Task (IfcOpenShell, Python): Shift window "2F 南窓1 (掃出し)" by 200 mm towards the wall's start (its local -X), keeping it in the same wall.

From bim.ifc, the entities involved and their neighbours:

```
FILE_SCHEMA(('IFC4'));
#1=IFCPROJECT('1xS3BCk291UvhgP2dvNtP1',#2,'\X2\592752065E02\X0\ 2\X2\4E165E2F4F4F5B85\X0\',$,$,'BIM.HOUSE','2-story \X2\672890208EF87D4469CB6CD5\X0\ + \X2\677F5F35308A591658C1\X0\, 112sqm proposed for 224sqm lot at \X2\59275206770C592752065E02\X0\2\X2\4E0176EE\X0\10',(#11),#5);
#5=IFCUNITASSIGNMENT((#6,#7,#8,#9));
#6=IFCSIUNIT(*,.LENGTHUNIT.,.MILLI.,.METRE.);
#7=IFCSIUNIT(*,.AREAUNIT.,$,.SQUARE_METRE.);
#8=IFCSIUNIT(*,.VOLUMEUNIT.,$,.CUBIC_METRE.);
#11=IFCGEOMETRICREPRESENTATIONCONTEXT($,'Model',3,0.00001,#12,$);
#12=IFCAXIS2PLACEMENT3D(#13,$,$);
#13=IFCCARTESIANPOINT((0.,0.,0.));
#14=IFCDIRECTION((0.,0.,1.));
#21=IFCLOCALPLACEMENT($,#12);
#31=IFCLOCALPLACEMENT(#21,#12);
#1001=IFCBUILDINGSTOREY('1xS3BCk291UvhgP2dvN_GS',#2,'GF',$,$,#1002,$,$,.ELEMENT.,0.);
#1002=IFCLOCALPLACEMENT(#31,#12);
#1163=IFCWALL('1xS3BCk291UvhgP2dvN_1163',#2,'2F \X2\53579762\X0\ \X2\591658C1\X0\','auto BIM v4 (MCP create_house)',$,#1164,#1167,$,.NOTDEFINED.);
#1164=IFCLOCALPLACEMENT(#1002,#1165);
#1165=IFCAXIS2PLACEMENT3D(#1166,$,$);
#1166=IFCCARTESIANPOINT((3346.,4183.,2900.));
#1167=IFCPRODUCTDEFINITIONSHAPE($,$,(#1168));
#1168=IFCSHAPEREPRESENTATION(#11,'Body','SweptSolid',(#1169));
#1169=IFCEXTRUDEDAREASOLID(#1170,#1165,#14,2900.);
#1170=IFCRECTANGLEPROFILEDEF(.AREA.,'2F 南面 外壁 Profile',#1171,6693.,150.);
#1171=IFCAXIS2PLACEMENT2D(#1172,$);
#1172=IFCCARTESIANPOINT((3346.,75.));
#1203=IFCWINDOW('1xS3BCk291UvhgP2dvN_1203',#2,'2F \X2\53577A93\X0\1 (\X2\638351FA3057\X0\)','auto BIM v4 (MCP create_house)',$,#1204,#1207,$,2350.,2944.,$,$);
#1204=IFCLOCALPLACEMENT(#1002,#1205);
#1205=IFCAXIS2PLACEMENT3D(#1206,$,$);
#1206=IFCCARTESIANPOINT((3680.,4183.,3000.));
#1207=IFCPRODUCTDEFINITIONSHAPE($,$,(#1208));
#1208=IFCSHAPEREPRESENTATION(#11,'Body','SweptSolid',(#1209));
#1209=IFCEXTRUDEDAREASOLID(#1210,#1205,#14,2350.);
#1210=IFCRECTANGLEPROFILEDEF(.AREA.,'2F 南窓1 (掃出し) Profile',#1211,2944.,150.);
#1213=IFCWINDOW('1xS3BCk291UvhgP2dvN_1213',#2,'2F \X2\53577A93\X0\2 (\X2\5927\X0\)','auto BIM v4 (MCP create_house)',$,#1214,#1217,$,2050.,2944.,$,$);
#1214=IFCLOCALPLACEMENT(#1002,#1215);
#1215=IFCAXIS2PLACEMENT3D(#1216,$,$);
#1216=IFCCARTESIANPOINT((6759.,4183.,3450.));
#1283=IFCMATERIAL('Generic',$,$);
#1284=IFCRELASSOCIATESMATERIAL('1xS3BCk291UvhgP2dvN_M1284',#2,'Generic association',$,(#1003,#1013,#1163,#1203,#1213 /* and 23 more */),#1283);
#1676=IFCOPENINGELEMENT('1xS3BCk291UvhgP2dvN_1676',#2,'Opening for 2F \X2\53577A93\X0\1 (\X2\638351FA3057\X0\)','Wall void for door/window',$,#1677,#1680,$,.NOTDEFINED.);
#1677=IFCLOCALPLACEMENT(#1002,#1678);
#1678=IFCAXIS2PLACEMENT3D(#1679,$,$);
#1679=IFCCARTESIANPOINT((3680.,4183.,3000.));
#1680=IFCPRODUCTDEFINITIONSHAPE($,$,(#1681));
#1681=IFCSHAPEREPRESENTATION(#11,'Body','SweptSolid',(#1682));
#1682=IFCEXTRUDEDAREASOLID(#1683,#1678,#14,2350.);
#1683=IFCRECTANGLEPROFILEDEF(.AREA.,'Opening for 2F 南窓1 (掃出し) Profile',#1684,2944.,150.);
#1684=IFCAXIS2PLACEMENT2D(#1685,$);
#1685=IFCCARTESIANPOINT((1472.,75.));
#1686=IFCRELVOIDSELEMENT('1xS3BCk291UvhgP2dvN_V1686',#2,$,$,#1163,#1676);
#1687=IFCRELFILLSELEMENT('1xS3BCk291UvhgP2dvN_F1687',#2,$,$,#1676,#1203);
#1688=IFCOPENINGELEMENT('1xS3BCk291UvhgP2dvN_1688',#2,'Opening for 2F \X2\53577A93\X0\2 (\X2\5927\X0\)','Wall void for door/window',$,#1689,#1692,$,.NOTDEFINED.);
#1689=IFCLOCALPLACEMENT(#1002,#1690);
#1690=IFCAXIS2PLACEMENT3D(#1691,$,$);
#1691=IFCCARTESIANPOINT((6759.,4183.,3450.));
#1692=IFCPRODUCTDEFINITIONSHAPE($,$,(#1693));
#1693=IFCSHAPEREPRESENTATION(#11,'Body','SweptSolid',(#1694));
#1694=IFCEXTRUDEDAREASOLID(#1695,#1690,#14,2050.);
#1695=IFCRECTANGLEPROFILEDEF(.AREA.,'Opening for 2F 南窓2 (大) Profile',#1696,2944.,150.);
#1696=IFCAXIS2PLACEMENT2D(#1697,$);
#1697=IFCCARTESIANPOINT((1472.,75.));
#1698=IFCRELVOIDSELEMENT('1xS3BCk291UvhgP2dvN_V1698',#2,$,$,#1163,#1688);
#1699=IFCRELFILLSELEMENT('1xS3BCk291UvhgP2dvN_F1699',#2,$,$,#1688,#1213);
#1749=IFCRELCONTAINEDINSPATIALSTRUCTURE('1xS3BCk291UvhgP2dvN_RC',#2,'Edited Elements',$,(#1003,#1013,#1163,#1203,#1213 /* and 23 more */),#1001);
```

```python
import ifcopenshell
import ifcopenshell.api.geometry
import ifcopenshell.util.placement
import ifcopenshell.util.unit

model = ifcopenshell.open("bim.ifc")
unit_scale = ifcopenshell.util.unit.calculate_unit_scale(model)

window = model.by_guid("1xS3BCk291UvhgP2dvN_1203")
opening = window.FillsVoids[0].RelatingOpeningElement
wall = opening.VoidsElements[0].RelatingBuildingElement

wall_matrix = ifcopenshell.util.placement.get_local_placement(wall.ObjectPlacement)
shift = wall_matrix[:3, 0] * -0.2 / unit_scale
before = ifcopenshell.util.placement.get_local_placement(window.ObjectPlacement)[:3, 3].copy()

# The window is not placed relative to its opening, so move both.
for product in (opening, window):
    matrix = ifcopenshell.util.placement.get_local_placement(product.ObjectPlacement)
    matrix[:3, 3] += shift
    ifcopenshell.api.geometry.edit_object_placement(model, product=product, matrix=matrix, is_si=False)

after = ifcopenshell.util.placement.get_local_placement(window.ObjectPlacement)[:3, 3]
print("window moved by", (after - before).round(3) + 0.0)

model.write("bim_edited.ifc")
```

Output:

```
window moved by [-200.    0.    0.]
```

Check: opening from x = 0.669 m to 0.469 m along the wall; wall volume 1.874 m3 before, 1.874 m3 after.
